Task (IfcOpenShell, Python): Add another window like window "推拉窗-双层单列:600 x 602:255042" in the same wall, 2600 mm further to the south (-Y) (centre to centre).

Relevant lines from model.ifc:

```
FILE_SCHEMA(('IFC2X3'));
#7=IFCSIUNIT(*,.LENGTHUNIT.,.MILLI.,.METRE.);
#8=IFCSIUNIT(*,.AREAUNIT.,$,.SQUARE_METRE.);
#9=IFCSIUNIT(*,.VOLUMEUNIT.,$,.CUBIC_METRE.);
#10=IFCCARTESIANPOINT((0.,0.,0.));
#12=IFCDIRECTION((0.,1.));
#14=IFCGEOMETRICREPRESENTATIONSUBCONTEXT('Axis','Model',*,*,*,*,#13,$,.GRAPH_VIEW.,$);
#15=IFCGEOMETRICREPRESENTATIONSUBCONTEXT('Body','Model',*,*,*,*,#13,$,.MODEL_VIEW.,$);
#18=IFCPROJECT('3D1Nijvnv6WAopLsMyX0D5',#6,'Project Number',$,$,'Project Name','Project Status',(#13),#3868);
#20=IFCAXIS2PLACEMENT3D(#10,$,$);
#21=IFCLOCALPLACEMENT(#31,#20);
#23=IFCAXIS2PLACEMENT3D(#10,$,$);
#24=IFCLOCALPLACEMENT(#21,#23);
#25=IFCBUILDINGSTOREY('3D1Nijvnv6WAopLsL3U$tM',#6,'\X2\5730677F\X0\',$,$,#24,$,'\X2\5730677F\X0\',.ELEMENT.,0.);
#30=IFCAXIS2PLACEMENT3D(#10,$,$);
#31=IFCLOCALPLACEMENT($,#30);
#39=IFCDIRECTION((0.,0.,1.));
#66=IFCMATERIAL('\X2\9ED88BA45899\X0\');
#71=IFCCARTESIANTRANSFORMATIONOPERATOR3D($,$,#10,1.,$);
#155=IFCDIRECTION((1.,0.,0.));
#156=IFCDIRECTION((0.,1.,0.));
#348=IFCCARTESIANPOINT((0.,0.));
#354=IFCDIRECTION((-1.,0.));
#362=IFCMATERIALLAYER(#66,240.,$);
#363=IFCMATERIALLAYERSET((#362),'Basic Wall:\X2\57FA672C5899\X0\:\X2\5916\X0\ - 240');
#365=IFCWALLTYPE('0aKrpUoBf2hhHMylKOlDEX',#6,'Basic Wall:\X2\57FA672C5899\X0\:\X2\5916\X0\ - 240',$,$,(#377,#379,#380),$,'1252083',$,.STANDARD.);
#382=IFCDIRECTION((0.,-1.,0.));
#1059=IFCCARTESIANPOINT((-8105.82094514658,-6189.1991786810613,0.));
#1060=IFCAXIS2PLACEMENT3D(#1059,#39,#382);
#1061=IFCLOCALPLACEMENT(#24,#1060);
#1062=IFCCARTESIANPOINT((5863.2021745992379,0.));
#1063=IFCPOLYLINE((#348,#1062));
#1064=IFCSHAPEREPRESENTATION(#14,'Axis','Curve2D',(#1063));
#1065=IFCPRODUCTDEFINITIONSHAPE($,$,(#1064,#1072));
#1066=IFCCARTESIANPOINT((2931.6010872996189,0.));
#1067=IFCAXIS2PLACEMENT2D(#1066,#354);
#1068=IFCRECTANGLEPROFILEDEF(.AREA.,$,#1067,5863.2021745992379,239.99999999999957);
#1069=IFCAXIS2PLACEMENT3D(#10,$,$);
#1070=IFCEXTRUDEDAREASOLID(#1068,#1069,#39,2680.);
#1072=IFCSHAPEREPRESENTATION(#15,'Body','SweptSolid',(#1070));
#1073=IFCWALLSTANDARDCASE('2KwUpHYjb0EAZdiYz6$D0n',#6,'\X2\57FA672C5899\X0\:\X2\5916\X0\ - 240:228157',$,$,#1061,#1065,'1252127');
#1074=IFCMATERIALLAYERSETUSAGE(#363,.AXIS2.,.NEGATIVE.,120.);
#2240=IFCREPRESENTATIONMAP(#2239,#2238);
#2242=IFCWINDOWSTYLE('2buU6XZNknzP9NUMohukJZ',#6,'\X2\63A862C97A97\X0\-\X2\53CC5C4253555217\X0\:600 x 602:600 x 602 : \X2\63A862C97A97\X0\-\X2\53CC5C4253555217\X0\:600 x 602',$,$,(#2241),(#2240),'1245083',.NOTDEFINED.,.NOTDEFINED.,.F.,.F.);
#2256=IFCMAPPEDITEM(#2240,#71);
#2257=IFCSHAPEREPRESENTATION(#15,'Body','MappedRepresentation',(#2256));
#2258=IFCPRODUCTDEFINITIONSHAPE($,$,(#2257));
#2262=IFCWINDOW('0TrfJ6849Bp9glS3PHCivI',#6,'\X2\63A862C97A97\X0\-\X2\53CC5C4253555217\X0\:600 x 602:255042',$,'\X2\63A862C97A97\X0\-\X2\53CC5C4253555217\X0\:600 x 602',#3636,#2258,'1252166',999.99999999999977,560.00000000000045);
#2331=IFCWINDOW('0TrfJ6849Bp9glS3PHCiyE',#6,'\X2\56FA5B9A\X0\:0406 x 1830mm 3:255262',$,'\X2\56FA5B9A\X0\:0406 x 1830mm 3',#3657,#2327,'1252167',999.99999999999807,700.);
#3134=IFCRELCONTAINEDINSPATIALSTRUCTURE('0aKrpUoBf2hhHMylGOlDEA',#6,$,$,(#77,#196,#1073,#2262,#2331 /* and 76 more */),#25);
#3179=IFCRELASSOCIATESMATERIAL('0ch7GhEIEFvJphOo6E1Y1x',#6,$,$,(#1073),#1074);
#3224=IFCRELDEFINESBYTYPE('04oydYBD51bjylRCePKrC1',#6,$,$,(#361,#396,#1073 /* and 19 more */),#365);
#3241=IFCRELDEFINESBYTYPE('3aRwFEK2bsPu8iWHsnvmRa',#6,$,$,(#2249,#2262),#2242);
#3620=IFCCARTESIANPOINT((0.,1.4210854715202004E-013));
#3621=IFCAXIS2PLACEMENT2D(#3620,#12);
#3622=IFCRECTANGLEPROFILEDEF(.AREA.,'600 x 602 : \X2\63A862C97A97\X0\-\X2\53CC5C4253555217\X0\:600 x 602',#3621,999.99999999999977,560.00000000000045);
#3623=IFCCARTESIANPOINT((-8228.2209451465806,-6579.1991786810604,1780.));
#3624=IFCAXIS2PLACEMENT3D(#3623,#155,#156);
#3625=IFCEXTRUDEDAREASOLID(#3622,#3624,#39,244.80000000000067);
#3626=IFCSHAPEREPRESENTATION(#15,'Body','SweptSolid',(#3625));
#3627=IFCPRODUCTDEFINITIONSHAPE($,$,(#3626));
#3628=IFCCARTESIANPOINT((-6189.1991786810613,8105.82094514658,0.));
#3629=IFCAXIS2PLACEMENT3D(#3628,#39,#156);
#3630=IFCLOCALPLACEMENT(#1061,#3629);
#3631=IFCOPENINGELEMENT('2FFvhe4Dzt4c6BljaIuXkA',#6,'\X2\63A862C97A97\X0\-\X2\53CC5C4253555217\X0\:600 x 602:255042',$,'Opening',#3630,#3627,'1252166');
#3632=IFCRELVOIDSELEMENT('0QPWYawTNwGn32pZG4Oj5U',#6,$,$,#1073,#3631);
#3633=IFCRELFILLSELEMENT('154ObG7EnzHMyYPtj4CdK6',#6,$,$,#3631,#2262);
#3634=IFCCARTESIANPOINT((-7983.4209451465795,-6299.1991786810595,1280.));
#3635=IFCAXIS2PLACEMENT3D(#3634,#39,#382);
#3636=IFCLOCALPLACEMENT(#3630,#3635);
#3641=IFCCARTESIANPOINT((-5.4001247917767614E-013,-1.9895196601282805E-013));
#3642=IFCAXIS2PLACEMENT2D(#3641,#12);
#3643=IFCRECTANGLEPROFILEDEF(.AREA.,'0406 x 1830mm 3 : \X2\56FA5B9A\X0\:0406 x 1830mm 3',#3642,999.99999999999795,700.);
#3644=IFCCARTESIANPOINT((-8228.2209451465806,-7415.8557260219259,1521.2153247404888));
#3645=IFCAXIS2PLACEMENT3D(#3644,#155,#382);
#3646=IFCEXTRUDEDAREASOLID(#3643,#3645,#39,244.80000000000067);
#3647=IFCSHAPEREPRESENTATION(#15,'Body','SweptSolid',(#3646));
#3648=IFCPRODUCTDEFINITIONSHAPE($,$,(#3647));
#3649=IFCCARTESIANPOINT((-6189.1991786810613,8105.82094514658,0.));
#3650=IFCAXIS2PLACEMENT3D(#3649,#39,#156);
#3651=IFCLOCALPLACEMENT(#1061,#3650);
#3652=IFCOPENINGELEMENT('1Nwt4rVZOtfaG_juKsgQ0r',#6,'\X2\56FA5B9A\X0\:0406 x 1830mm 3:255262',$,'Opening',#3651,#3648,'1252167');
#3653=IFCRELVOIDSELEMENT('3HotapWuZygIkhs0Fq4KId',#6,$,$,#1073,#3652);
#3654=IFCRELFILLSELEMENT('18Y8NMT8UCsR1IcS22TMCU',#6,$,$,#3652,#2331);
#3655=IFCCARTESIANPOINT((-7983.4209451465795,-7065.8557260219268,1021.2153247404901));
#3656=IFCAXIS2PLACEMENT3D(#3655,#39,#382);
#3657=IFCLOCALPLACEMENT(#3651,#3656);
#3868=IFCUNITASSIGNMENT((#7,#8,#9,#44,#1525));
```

```python
import ifcopenshell
import ifcopenshell.api.feature
import ifcopenshell.api.geometry
import ifcopenshell.api.root
import ifcopenshell.geom
import ifcopenshell.util.element
import ifcopenshell.util.placement
import ifcopenshell.util.shape
import ifcopenshell.util.unit

model = ifcopenshell.open("model.ifc")
unit_scale = ifcopenshell.util.unit.calculate_unit_scale(model)
settings = ifcopenshell.geom.settings()


def volume(element):
    """Net volume in cubic metres, openings subtracted."""
    shape = ifcopenshell.geom.create_shape(settings, element)
    return ifcopenshell.util.shape.get_volume(shape.geometry)


def reuse_history(source, copy):
    """copy_class also copies each property set's owner history, people and application; keep the originals."""
    for rel in copy.IsDefinedBy:
        if rel.is_a("IfcRelDefinesByProperties") and (history := rel.RelatingPropertyDefinition.OwnerHistory):
            rel.RelatingPropertyDefinition.OwnerHistory = source.OwnerHistory
            ifcopenshell.util.element.remove_deep2(model, history)


window = model.by_guid("0TrfJ6849Bp9glS3PHCivI")
opening = window.FillsVoids[0].RelatingOpeningElement
wall = opening.VoidsElements[0].RelatingBuildingElement
before = volume(wall)
shift = ifcopenshell.util.placement.get_local_placement(wall.ObjectPlacement)[:3, 0] * 2.6 / unit_scale

# copy_class copies the void relationship, type, container and properties, but no geometry.
new_opening = ifcopenshell.api.root.copy_class(model, product=opening)
new_opening.Representation = ifcopenshell.util.element.copy_deep(
    model, opening.Representation, exclude=["IfcGeometricRepresentationContext", "IfcRepresentationMap"]
)
new_opening.Name = "推拉窗-双层单列:600 x 602"
new_opening.Tag = None
new_window = ifcopenshell.api.root.copy_class(model, product=window)
new_window.Representation = ifcopenshell.util.element.copy_deep(
    model, window.Representation, exclude=["IfcGeometricRepresentationContext", "IfcRepresentationMap"]
)
new_window.Name = "推拉窗-双层单列:600 x 602"
new_window.Tag = None
reuse_history(window, new_window)
fills = ifcopenshell.api.feature.add_filling(model, opening=new_opening, element=new_window)
fills.OwnerHistory = new_window.OwnerHistory  # required in IFC2X3

for old, new in ((opening, new_opening), (window, new_window)):
    matrix = ifcopenshell.util.placement.get_local_placement(old.ObjectPlacement)
    matrix[:3, 3] += shift
    ifcopenshell.api.geometry.edit_object_placement(model, product=new, matrix=matrix, is_si=False)

after = volume(wall)

print(f"wall volume {before:.3f} -> {after:.3f} m3")

model.write("model-out.ifc")
```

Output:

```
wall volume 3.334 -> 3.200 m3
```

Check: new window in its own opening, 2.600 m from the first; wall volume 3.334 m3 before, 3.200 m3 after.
